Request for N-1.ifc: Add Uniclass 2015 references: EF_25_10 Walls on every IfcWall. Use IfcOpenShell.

First a look at what the model holds.

```python
import ifcopenshell

model = ifcopenshell.open("N-1.ifc")
print(model.schema)
print("classifications:", [c.Name for c in model.by_type("IfcClassification")])
for ifc_class in ("IfcDoor", "IfcRoof", "IfcStair", "IfcWall", "IfcWindow"):
    print(ifc_class, len(model.by_type(ifc_class)))
```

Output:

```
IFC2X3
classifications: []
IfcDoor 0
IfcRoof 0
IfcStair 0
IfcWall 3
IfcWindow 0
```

```python
import ifcopenshell
import ifcopenshell.api.classification

model = ifcopenshell.open("N-1.ifc")

# IFC2X3 requires Source and Edition and has no link from the project to the system.
system = model.create_entity("IfcClassification", Source="NBS", Edition="2015", Name="Uniclass 2015")

codes = {
    "IfcWall": ("EF_25_10", "Walls"),
}
for ifc_class, (code, name) in codes.items():
    products = model.by_type(ifc_class)
    ifcopenshell.api.classification.add_reference(
        model, products=products, classification=system, identification=code, name=name
    )
    print(code, len(products))

model.write("N-1_v2.ifc")
```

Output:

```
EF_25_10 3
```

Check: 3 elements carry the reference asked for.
